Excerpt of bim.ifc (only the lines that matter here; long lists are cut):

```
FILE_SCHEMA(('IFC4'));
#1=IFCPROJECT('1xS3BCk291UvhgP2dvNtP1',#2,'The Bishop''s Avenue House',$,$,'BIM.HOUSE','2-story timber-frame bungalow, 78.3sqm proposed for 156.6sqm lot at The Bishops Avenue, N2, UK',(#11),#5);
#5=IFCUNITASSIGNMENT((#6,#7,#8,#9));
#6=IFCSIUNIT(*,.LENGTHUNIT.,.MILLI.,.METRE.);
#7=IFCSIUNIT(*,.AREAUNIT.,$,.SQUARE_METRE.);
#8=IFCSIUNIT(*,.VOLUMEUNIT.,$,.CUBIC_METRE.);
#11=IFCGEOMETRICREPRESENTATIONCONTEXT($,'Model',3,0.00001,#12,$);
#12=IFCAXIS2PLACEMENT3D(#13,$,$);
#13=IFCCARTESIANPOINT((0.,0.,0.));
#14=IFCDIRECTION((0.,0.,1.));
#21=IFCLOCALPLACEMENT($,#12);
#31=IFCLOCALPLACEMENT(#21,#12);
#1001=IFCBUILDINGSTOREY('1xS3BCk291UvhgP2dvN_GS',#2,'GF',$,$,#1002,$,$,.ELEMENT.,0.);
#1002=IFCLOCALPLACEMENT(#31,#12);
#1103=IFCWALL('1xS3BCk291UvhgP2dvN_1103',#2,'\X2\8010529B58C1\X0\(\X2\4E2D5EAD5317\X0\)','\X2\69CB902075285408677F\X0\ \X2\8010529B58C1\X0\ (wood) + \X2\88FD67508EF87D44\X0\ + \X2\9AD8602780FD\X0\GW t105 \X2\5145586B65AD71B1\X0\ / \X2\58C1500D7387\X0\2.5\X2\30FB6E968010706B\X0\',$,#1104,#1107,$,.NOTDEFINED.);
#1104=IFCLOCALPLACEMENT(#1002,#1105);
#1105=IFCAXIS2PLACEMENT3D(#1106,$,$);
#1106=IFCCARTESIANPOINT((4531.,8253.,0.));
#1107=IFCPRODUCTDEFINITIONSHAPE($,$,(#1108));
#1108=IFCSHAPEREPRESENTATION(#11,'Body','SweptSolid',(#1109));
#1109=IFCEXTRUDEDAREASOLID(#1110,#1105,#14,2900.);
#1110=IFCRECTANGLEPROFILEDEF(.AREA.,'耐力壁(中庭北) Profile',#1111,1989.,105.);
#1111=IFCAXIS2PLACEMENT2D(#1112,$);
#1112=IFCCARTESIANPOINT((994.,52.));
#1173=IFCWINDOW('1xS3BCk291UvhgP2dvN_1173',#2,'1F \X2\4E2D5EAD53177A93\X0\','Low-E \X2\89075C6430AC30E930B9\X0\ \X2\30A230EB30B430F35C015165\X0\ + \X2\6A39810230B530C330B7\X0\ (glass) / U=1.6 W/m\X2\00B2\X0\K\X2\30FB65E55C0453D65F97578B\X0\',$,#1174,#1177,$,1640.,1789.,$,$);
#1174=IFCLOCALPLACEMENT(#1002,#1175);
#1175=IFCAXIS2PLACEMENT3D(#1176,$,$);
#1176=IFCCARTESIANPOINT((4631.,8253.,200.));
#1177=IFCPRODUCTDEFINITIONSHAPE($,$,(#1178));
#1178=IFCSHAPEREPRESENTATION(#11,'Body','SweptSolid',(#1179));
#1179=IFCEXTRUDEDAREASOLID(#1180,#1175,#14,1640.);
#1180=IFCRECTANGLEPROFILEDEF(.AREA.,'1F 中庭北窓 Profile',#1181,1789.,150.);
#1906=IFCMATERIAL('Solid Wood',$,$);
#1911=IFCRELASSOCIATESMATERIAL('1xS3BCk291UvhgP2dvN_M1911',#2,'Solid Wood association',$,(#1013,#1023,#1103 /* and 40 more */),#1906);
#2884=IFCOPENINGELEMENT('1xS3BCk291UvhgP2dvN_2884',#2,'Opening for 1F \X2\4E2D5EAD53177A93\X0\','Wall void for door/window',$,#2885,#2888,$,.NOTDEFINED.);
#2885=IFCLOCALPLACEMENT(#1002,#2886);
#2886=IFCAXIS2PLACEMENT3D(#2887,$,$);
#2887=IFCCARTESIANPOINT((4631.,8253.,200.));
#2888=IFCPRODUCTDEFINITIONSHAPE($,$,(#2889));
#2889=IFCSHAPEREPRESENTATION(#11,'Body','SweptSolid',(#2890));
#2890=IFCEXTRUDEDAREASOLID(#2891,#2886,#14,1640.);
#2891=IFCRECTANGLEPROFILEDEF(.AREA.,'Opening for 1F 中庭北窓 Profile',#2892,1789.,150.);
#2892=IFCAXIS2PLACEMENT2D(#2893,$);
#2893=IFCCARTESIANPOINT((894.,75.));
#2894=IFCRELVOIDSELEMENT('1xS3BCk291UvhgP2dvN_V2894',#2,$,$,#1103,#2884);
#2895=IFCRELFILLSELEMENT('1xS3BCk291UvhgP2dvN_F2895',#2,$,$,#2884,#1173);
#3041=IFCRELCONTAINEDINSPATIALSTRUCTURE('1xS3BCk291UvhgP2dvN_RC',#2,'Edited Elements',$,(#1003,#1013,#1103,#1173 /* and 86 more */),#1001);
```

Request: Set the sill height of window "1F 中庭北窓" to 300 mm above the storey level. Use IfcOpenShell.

```python
import numpy as np
import ifcopenshell
import ifcopenshell.api.geometry
import ifcopenshell.geom
import ifcopenshell.util.element
import ifcopenshell.util.placement
import ifcopenshell.util.shape
import ifcopenshell.util.unit

model = ifcopenshell.open("bim.ifc")
unit_scale = ifcopenshell.util.unit.calculate_unit_scale(model)

window = model.by_id(1173)
opening = window.FillsVoids[0].RelatingOpeningElement
storey = ifcopenshell.util.element.get_container(window, ifc_class="IfcBuildingStorey")
level = ifcopenshell.util.placement.get_local_placement(storey.ObjectPlacement)[2, 3]

# The opening's origin need not be at the sill, so measure its lowest point.
shape = ifcopenshell.geom.create_shape(ifcopenshell.geom.settings(), opening)
bottom = ifcopenshell.util.shape.get_shape_bottom_elevation(shape, shape.geometry) / unit_scale
dz = level + 0.3 / unit_scale - bottom

shift = np.array([0.0, 0.0, dz])
# The window is not placed relative to its opening, so move both.
for product in (opening, window):
    matrix = ifcopenshell.util.placement.get_local_placement(product.ObjectPlacement)
    matrix[:3, 3] += shift
    ifcopenshell.api.geometry.edit_object_placement(model, product=product, matrix=matrix, is_si=False)

print(f"moved by {dz * unit_scale:+.3f} m")

model.write("bim-out.ifc")
```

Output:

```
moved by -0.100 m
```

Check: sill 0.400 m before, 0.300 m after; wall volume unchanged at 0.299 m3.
